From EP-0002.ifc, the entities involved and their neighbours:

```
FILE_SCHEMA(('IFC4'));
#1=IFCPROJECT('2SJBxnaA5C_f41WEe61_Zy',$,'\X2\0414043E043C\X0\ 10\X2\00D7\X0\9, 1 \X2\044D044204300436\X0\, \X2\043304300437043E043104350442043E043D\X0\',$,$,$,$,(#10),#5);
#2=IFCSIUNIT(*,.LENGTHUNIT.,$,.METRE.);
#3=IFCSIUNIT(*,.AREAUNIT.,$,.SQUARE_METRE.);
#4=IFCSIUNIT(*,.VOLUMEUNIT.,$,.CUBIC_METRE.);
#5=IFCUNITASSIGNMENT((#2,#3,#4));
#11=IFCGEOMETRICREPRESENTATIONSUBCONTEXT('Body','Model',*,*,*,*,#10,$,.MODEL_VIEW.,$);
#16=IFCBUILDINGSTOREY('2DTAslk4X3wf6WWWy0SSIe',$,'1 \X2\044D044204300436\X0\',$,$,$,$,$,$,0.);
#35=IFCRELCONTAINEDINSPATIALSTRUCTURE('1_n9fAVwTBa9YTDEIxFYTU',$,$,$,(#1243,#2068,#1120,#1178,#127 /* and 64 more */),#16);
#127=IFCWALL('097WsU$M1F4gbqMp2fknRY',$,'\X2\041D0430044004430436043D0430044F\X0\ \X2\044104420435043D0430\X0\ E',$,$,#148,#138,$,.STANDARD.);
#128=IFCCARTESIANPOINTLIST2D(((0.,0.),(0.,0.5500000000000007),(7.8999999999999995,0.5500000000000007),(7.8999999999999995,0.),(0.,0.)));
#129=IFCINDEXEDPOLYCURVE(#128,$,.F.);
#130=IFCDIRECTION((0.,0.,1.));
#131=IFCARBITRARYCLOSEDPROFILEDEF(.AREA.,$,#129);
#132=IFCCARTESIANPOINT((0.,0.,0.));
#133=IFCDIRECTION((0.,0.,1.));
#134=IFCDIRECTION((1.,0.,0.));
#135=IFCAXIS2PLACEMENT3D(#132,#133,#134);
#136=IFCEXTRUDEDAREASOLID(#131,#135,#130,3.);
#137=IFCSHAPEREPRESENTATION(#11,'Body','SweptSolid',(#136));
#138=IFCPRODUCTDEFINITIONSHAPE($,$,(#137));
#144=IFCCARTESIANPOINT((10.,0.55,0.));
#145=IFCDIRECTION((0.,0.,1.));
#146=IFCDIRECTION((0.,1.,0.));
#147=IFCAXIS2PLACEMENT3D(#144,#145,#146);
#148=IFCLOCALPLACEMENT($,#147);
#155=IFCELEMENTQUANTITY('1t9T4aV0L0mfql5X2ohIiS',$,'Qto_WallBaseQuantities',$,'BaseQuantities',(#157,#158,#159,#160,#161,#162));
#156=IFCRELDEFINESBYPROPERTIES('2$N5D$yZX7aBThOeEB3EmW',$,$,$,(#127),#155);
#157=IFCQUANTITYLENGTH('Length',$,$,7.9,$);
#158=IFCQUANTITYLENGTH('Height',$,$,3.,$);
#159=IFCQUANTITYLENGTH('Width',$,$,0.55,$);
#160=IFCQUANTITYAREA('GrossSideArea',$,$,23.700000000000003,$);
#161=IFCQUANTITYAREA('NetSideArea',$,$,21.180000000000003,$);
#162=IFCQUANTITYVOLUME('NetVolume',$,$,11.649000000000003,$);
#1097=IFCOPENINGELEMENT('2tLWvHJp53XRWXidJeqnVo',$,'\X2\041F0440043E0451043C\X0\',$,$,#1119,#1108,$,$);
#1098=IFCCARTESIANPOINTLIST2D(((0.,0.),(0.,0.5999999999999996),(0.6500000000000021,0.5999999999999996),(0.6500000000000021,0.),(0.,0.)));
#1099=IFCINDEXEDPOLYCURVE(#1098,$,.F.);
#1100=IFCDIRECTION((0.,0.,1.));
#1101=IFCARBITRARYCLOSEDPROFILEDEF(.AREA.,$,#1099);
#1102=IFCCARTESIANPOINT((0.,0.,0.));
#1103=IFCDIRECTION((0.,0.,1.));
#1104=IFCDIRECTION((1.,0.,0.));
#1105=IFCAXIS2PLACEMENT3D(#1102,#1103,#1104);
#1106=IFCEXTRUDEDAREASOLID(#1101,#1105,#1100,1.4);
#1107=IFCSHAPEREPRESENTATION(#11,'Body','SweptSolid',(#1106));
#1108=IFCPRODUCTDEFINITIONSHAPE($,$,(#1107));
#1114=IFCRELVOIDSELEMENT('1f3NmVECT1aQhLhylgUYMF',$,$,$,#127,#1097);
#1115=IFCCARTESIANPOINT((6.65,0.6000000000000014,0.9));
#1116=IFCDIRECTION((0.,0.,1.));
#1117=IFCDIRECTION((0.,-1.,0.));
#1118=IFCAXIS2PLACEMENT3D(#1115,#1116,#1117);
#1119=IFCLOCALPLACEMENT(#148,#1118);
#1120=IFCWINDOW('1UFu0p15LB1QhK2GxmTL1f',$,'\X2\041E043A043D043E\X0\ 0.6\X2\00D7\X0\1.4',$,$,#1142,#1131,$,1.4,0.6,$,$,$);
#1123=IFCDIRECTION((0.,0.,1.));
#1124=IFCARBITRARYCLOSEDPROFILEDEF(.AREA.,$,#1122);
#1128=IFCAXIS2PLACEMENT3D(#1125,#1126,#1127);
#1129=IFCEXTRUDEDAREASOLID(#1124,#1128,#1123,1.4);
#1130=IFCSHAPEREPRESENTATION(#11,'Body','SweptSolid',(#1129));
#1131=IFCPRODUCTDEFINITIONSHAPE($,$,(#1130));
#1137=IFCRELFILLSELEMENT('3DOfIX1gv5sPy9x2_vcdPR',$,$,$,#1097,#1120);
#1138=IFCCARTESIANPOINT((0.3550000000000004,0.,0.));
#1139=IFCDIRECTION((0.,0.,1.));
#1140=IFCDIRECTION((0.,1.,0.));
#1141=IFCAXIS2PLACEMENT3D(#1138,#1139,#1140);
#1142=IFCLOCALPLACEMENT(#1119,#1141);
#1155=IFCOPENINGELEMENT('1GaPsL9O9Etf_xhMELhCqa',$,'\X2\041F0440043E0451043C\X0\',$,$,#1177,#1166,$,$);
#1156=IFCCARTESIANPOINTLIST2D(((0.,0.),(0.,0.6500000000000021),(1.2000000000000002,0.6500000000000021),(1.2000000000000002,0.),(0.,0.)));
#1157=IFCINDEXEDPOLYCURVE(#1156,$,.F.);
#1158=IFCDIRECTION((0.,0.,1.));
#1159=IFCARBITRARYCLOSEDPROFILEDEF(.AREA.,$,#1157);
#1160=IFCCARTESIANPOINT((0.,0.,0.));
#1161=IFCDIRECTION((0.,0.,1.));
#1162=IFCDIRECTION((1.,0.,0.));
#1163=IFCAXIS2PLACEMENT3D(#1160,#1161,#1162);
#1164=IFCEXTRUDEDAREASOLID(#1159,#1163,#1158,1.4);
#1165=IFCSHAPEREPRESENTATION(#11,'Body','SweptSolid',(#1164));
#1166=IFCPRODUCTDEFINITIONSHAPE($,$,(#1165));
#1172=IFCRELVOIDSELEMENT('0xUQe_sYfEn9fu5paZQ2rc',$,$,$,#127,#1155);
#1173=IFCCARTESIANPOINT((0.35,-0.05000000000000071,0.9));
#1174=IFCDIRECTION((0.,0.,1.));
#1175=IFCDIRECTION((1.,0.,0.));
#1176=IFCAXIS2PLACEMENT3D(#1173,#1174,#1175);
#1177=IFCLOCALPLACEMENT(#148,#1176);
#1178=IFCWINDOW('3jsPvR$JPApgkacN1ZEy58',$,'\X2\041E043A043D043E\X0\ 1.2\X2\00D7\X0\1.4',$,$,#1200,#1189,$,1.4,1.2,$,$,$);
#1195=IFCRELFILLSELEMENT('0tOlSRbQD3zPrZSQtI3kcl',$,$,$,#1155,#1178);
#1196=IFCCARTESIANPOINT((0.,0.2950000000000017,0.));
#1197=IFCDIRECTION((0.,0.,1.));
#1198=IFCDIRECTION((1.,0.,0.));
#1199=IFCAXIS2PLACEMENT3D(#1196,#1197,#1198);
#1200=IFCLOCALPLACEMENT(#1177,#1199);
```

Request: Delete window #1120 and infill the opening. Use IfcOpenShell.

```python
import ifcopenshell
import ifcopenshell.api.feature
import ifcopenshell.api.pset
import ifcopenshell.api.root
import ifcopenshell.geom
import ifcopenshell.util.element
import ifcopenshell.util.shape
import ifcopenshell.util.unit

model = ifcopenshell.open("EP-0002.ifc")
area_scale = ifcopenshell.util.unit.calculate_unit_scale(model, "AREAUNIT")
volume_scale = ifcopenshell.util.unit.calculate_unit_scale(model, "VOLUMEUNIT")
settings = ifcopenshell.geom.settings()


def volume(element):
    """Net volume in cubic metres, openings subtracted."""
    shape = ifcopenshell.geom.create_shape(settings, element)
    return ifcopenshell.util.shape.get_volume(shape.geometry)


window = model.by_guid("1UFu0p15LB1QhK2GxmTL1f")
opening = window.FillsVoids[0].RelatingOpeningElement
wall = opening.VoidsElements[0].RelatingBuildingElement
before = volume(wall)

ifcopenshell.api.root.remove_product(model, product=window)
ifcopenshell.api.feature.remove_feature(model, feature=opening)

after = volume(wall)
thickness = 0.55  # wall thickness in metres

# Update the wall's stored quantities.
qto = model.by_id(ifcopenshell.util.element.get_pset(wall, "Qto_WallBaseQuantities", should_inherit=False)["id"])
ifcopenshell.api.pset.edit_qto(model, qto=qto, properties={
    "NetSideArea": after / thickness / area_scale,
    "NetVolume": after / volume_scale,
})

print(f"wall volume {before:.3f} -> {after:.3f} m3")

model.write("EP-0002_updated.ifc")
```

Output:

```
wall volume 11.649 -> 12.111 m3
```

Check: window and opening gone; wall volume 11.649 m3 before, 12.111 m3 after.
